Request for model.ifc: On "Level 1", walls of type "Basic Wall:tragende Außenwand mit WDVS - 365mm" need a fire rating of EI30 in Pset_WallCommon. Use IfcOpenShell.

First a look at what the model holds.

```python
import ifcopenshell
import ifcopenshell.util.element

model = ifcopenshell.open("model.ifc")
print(model.schema)
storey = next(s for s in model.by_type("IfcBuildingStorey") if s.Name == "Level 1")
walls = [e for e in ifcopenshell.util.element.get_decomposition(storey) if e.is_a("IfcWall")]
seen = {}
for e in walls:
    element_type = ifcopenshell.util.element.get_type(e)
    key = (element_type.Name if element_type != e and element_type else None, ifcopenshell.util.element.get_pset(e, "Pset_WallCommon", "FireRating"))
    seen[key] = seen.get(key, 0) + 1
for (name, value), count in sorted(seen.items(), key=str):
    print(count, "x", name, "|", value)
```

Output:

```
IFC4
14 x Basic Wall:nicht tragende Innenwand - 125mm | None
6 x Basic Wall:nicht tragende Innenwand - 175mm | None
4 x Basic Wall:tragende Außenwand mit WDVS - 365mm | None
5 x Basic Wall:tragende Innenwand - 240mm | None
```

```python
import ifcopenshell
import ifcopenshell.api.pset
import ifcopenshell.util.element

model = ifcopenshell.open("model.ifc")

storey = next(s for s in model.by_type("IfcBuildingStorey") if s.Name == "Level 1")
walls = [e for e in ifcopenshell.util.element.get_decomposition(storey) if e.is_a("IfcWall")]

count = 0
for e in walls:
    element_type = ifcopenshell.util.element.get_type(e)
    if element_type in (None, e) or element_type.Name != "Basic Wall:tragende Außenwand mit WDVS - 365mm":
        continue
    # add_pset returns the element's existing set when there is one.
    pset = ifcopenshell.api.pset.add_pset(model, product=e, name="Pset_WallCommon")
    ifcopenshell.api.pset.edit_pset(model, pset=pset, properties={"FireRating": "EI30"})
    count += 1

print(count, "walls updated")

model.write("model_updated.ifc")
```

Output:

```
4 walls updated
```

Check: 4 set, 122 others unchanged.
